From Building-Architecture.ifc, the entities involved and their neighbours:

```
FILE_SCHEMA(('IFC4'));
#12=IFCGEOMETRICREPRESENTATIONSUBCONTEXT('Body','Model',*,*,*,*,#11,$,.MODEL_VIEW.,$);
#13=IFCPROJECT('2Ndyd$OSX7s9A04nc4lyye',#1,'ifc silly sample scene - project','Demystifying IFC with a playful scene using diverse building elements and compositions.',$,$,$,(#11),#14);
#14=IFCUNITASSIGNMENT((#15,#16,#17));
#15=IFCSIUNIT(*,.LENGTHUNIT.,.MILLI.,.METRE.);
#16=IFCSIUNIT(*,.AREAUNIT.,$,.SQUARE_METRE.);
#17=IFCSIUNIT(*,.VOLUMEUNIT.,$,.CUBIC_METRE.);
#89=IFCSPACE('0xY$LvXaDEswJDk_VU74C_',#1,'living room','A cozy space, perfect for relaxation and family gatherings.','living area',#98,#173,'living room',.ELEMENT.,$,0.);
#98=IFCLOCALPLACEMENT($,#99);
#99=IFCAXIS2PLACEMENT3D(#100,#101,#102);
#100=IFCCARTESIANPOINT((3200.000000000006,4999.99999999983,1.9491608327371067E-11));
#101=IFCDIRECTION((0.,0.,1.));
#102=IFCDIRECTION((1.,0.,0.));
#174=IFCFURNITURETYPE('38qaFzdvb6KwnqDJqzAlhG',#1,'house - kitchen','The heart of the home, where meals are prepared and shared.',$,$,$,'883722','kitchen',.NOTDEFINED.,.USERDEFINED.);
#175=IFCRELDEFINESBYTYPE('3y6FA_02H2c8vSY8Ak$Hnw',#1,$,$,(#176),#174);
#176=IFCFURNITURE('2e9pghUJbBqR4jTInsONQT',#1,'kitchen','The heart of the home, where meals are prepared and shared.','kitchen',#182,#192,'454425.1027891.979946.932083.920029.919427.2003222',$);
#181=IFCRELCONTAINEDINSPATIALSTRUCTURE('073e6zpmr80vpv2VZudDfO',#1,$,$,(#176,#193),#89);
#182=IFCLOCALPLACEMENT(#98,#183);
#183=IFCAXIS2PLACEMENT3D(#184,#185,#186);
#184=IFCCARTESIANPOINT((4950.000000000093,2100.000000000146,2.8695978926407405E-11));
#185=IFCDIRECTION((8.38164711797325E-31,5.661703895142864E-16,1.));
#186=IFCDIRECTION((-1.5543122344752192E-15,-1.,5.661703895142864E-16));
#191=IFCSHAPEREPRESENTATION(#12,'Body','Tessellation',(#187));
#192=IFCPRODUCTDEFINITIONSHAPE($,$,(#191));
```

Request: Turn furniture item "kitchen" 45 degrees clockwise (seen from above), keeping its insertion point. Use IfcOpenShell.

```python
import ifcopenshell
import ifcopenshell.api.geometry
import ifcopenshell.util.placement

model = ifcopenshell.open("Building-Architecture.ifc")

item = model.by_id(176)
matrix = ifcopenshell.util.placement.get_local_placement(item.ObjectPlacement)
matrix = matrix @ ifcopenshell.util.placement.rotation(-45, "Z")
ifcopenshell.api.geometry.edit_object_placement(model, product=item, matrix=matrix, is_si=False)

print(ifcopenshell.util.placement.get_local_placement(item.ObjectPlacement).round(3) + 0.0)

model.write("Building-Architecture_updated.ifc")
```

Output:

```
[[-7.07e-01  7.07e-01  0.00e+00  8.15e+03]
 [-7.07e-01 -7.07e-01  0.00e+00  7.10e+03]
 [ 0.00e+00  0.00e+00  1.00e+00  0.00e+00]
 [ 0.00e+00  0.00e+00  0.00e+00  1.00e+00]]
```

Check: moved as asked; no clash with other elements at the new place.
